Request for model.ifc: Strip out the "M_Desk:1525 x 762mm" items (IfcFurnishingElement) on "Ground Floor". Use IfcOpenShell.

First a look at what the model holds.

```python
import ifcopenshell
import ifcopenshell.util.element

model = ifcopenshell.open("model.ifc")
print(model.schema)
storey = next(s for s in model.by_type("IfcBuildingStorey") if s.Name == "Ground Floor")
furniture = [e for e in ifcopenshell.util.element.get_decomposition(storey) if e.is_a("IfcFurnishingElement")]
seen = {}
for e in furniture:
    element_type = ifcopenshell.util.element.get_type(e)
    name = element_type.Name if element_type not in (None, e) else None
    seen[name] = seen.get(name, 0) + 1
for name, count in sorted(seen.items(), key=str):
    print(count, "x", name)
```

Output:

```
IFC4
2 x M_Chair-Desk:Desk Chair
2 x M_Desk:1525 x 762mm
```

```python
import ifcopenshell
import ifcopenshell.api.root
import ifcopenshell.util.element

model = ifcopenshell.open("model.ifc")

storey = next(s for s in model.by_type("IfcBuildingStorey") if s.Name == "Ground Floor")
furniture = [e for e in ifcopenshell.util.element.get_decomposition(storey) if e.is_a("IfcFurnishingElement")]
targets = [e for e in furniture if (t := ifcopenshell.util.element.get_type(e)) not in (None, e) and t.Name == "M_Desk:1525 x 762mm"]

for e in targets:
    ifcopenshell.api.root.remove_product(model, product=e)
print(len(targets), "removed")

model.write("model_edited.ifc")
```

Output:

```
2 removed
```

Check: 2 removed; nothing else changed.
